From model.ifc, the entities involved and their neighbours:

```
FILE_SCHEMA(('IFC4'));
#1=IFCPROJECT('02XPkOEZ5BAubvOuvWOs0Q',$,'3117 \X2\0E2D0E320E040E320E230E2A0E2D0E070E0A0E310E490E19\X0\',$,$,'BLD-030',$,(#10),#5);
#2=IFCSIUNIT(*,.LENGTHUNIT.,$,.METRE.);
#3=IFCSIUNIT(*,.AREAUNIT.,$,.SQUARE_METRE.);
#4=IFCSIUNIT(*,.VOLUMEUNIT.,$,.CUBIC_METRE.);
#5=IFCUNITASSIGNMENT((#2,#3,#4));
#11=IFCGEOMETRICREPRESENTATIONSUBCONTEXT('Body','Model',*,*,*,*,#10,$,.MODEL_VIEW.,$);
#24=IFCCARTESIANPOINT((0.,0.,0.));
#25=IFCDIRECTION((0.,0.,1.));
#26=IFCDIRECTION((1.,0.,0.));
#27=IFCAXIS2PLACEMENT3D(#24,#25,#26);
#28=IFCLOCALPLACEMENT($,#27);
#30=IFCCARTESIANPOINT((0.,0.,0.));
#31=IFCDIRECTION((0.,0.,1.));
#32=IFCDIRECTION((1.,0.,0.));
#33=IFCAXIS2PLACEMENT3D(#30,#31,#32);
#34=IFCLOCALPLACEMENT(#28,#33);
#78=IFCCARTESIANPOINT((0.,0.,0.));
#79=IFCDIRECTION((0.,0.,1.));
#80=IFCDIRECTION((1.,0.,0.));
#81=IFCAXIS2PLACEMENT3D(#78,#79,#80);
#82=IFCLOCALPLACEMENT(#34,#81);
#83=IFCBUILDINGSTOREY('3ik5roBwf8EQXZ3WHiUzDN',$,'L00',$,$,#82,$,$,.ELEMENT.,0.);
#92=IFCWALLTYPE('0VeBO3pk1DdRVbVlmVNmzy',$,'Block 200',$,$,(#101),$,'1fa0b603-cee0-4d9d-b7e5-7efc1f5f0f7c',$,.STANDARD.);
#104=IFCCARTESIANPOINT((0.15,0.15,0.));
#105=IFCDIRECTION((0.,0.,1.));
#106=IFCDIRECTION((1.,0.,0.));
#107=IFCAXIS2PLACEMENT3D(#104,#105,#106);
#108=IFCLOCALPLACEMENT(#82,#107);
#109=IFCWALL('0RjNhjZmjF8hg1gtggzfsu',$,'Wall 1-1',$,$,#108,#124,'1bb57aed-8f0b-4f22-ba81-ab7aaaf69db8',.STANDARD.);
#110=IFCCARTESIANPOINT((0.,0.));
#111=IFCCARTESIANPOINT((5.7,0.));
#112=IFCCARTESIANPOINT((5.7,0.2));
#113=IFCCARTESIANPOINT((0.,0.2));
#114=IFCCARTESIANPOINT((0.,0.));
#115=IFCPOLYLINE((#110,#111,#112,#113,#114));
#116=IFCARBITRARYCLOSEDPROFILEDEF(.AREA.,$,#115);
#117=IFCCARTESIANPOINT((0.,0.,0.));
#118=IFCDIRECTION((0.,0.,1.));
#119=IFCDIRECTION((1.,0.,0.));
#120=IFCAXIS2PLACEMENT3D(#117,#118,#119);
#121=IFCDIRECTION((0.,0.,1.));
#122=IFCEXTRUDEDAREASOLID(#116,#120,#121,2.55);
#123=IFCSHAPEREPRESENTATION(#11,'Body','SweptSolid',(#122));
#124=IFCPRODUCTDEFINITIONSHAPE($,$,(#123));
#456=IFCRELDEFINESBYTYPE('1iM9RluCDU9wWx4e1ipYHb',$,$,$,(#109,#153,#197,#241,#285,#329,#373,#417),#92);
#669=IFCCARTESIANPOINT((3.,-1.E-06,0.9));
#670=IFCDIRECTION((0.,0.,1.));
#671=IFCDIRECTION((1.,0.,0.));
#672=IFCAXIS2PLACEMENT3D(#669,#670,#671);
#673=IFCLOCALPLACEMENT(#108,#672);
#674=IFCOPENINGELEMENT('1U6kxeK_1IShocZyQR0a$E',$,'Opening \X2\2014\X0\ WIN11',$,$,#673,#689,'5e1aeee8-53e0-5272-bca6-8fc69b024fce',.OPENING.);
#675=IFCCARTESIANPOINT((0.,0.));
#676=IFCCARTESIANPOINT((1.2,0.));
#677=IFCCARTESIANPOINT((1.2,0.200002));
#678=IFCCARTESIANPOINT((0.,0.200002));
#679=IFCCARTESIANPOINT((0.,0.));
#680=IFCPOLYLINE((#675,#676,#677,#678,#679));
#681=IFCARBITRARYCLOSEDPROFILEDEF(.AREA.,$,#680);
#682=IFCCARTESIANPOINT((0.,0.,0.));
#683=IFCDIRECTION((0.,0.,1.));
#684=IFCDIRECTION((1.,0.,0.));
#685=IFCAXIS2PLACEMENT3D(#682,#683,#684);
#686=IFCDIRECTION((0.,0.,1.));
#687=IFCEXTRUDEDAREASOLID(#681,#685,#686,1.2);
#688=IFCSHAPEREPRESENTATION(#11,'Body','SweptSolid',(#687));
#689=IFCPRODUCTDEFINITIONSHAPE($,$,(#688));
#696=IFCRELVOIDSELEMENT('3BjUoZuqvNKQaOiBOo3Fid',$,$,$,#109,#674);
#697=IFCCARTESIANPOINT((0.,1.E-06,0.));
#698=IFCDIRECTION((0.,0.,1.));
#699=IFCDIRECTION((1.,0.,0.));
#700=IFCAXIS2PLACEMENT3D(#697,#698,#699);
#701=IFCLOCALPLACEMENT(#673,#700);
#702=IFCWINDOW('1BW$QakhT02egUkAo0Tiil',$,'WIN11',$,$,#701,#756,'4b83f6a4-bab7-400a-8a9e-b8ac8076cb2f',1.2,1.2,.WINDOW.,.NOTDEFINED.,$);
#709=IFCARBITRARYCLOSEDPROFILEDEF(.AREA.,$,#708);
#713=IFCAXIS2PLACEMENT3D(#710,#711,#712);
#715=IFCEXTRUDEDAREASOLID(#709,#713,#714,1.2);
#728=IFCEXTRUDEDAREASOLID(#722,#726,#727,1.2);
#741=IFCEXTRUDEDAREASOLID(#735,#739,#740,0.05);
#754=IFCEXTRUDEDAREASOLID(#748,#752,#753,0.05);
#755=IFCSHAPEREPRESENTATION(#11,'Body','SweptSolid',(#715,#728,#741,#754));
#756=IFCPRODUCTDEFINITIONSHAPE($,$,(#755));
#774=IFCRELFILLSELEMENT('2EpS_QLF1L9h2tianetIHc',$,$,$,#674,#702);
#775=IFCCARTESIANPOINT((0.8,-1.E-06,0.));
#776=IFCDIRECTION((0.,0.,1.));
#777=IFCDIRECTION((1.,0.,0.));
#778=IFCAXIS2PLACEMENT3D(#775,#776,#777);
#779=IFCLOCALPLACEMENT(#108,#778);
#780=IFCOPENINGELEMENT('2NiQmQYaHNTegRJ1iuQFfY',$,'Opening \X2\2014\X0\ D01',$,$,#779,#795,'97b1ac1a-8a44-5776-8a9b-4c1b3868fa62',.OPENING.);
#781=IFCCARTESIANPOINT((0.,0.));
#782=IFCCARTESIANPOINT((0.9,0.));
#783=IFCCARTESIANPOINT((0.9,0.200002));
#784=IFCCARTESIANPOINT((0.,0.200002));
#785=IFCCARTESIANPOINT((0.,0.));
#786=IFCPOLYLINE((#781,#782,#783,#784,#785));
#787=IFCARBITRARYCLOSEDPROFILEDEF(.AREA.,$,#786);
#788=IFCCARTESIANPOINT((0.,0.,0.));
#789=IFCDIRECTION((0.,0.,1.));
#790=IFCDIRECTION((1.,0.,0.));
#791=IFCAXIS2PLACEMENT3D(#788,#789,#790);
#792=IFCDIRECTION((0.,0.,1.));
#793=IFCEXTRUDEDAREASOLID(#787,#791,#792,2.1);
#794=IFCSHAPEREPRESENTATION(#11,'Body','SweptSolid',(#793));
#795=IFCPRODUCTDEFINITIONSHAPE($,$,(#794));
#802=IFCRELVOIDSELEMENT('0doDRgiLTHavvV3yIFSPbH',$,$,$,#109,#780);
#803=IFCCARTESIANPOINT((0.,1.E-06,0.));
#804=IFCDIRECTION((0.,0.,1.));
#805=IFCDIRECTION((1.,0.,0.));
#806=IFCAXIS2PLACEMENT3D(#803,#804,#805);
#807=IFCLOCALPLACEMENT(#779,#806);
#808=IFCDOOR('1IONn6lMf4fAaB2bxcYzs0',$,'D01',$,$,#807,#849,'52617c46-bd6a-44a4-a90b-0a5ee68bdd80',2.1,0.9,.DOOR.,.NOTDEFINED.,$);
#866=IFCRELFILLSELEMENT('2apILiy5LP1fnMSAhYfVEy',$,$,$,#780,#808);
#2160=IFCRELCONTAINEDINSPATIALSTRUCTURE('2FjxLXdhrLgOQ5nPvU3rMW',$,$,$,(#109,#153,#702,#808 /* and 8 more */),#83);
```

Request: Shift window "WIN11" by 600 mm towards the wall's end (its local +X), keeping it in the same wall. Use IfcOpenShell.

```python
import ifcopenshell
import ifcopenshell.api.geometry
import ifcopenshell.util.placement

model = ifcopenshell.open("model.ifc")

window = model.by_guid("1BW$QakhT02egUkAo0Tiil")
opening = window.FillsVoids[0].RelatingOpeningElement
wall = opening.VoidsElements[0].RelatingBuildingElement

wall_matrix = ifcopenshell.util.placement.get_local_placement(wall.ObjectPlacement)
shift = wall_matrix[:3, 0] * 0.6
before = ifcopenshell.util.placement.get_local_placement(window.ObjectPlacement)[:3, 3].copy()

# The window is placed relative to its opening, so it follows when the opening moves.
matrix = ifcopenshell.util.placement.get_local_placement(opening.ObjectPlacement)
matrix[:3, 3] += shift
ifcopenshell.api.geometry.edit_object_placement(
    model, product=opening, matrix=matrix, is_si=False, should_transform_children=True
)

after = ifcopenshell.util.placement.get_local_placement(window.ObjectPlacement)[:3, 3]
print("window moved by", (after - before).round(3) + 0.0)

model.write("model_edited.ifc")
```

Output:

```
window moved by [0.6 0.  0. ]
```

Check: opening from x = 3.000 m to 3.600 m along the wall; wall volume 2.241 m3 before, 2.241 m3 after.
